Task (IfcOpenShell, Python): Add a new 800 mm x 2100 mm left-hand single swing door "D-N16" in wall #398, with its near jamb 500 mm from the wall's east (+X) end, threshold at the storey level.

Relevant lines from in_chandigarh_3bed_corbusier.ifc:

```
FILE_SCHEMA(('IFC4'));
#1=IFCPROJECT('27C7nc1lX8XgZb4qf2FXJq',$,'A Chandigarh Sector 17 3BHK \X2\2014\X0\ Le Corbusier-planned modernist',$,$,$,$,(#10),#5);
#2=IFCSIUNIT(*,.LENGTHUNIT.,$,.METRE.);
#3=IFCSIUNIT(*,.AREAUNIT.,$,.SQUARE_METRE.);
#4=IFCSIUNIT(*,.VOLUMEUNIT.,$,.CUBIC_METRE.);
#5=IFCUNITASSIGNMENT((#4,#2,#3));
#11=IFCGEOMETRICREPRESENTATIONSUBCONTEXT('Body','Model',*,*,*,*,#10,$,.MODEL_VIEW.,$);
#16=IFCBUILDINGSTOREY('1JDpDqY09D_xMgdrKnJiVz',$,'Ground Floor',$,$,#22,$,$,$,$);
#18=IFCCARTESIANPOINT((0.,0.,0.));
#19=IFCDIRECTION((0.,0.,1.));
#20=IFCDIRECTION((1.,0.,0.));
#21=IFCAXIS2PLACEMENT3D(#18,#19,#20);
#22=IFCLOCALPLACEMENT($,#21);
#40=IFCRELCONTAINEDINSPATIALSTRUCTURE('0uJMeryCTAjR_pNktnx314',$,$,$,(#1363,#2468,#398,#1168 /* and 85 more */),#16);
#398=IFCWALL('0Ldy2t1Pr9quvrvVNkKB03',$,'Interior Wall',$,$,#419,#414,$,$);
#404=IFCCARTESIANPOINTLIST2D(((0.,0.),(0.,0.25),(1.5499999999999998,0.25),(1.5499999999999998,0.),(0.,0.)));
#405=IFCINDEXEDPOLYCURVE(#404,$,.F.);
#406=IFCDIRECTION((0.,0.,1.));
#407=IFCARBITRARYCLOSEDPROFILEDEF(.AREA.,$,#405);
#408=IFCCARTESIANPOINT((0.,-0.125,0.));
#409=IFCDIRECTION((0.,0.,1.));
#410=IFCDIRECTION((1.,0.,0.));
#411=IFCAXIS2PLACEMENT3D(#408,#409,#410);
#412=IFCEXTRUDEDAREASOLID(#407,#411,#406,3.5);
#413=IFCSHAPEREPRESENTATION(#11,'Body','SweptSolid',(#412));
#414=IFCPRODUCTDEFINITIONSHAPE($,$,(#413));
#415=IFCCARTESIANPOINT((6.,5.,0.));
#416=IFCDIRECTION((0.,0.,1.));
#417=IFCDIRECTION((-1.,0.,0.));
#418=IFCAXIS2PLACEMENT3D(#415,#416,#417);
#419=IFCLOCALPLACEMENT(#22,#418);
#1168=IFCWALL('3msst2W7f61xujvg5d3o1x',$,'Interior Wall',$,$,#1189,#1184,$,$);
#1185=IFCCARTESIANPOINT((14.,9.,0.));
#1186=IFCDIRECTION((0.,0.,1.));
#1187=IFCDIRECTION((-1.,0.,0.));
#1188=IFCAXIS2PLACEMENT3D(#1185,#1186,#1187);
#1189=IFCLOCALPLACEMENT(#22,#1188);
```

```python
import numpy as np
import ifcopenshell
import ifcopenshell.api.feature
import ifcopenshell.api.geometry
import ifcopenshell.api.root
import ifcopenshell.api.spatial
import ifcopenshell.geom
import ifcopenshell.util.element
import ifcopenshell.util.placement
import ifcopenshell.util.representation
import ifcopenshell.util.shape
import ifcopenshell.util.unit

model = ifcopenshell.open("in_chandigarh_3bed_corbusier.ifc")
unit_scale = ifcopenshell.util.unit.calculate_unit_scale(model)
settings = ifcopenshell.geom.settings()


def volume(element):
    """Net volume in cubic metres, openings subtracted."""
    shape = ifcopenshell.geom.create_shape(settings, element)
    return ifcopenshell.util.shape.get_volume(shape.geometry)


wall = model.by_id(398)
storey = ifcopenshell.util.element.get_container(wall, ifc_class="IfcBuildingStorey")
context = ifcopenshell.util.representation.get_context(model, "Model", "Body", "MODEL_VIEW")
before = volume(wall)

width, height, from_end, sill = 0.8, 2.1, 0.5, 0.0  # metres

# The wall runs along its own X axis, and the end named is its -X end.
wall_shape = ifcopenshell.geom.create_shape(settings, wall)
x, y, z = ifcopenshell.util.shape.get_vertices(wall_shape.geometry).T
start = x.min() + from_end
face, thickness = float(y.min()), float(y.max() - y.min())
wall_matrix = ifcopenshell.util.placement.get_local_placement(wall.ObjectPlacement)
level = ifcopenshell.util.placement.get_local_placement(storey.ObjectPlacement)[2, 3]


def in_wall(x, y):
    """Placement at x, y metres in the wall's axes, at sill height."""
    matrix = wall_matrix.copy()
    matrix[:, 3] = wall_matrix @ np.array([x / unit_scale, y / unit_scale, 0.0, 1.0])
    matrix[2, 3] = level + sill / unit_scale
    return matrix


# Opening: a box that overshoots both wall faces by 50 mm.
opening = ifcopenshell.api.root.create_entity(model, ifc_class="IfcOpeningElement", predefined_type="OPENING")
box = ifcopenshell.api.geometry.add_wall_representation(
    model, context=context, length=width, height=height, thickness=thickness + 0.1
)
ifcopenshell.api.geometry.assign_representation(model, product=opening, representation=box)
ifcopenshell.api.geometry.edit_object_placement(model, product=opening, matrix=in_wall(start, face - 0.05), is_si=False)
ifcopenshell.api.feature.add_feature(model, feature=opening, element=wall)

door = ifcopenshell.api.root.create_entity(model, ifc_class="IfcDoor", name="D-N16", predefined_type="DOOR")
door.OverallWidth, door.OverallHeight = width / unit_scale, height / unit_scale
door.OperationType = "SINGLE_SWING_LEFT"
body = ifcopenshell.api.geometry.add_door_representation(
    model,
    context=context,
    overall_width=door.OverallWidth,
    overall_height=door.OverallHeight,
    operation_type="SINGLE_SWING_LEFT",
    lining_properties={"LiningDepth": thickness / unit_scale, "ThresholdDepth": thickness / unit_scale},
)
ifcopenshell.api.geometry.assign_representation(model, product=door, representation=body)
ifcopenshell.api.spatial.assign_container(model, products=[door], relating_structure=storey)
ifcopenshell.api.feature.add_filling(model, opening=opening, element=door)

# The lining spans the wall, so the door starts at the wall face.
ifcopenshell.api.geometry.edit_object_placement(model, product=door, matrix=in_wall(start, face), is_si=False)

after = volume(wall)

print(f"wall volume {before:.3f} -> {after:.3f} m3")

model.write("in_chandigarh_3bed_corbusier_rev.ifc")
```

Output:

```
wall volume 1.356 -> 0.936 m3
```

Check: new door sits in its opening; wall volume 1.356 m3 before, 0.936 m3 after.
